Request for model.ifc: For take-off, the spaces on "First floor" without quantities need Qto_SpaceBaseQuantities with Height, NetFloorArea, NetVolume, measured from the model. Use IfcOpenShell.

First a look at what the model holds.

```python
import ifcopenshell
import ifcopenshell.util.element
import ifcopenshell.util.unit

model = ifcopenshell.open("model.ifc")
print(model.schema)
for unit_type in ("LENGTHUNIT", "AREAUNIT", "VOLUMEUNIT"):
    print(unit_type, ifcopenshell.util.unit.calculate_unit_scale(model, unit_type))
storey = next(s for s in model.by_type("IfcBuildingStorey") if s.Name == "First floor")
spaces = [e for e in ifcopenshell.util.element.get_decomposition(storey) if e.is_a("IfcSpace")]
for e in sorted(spaces, key=lambda e: e.id()):
    print(e.id(), e.is_a(), e.Name, list(ifcopenshell.util.element.get_psets(e, qtos_only=True)), sep=" | ")
```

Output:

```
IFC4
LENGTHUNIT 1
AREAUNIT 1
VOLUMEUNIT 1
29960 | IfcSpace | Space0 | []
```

```python
import ifcopenshell
import ifcopenshell.api.pset
import ifcopenshell.geom
import ifcopenshell.util.element
import ifcopenshell.util.shape
import ifcopenshell.util.unit

model = ifcopenshell.open("model.ifc")
unit_scale = ifcopenshell.util.unit.calculate_unit_scale(model)
area_scale = ifcopenshell.util.unit.calculate_unit_scale(model, "AREAUNIT")
volume_scale = ifcopenshell.util.unit.calculate_unit_scale(model, "VOLUMEUNIT")
settings = ifcopenshell.geom.settings()

storey = next(s for s in model.by_type("IfcBuildingStorey") if s.Name == "First floor")
spaces = [e for e in ifcopenshell.util.element.get_decomposition(storey) if e.is_a("IfcSpace")]

for e in sorted(spaces, key=lambda e: e.id()):
    if ifcopenshell.util.element.get_psets(e, qtos_only=True, should_inherit=False):
        continue
    # Geometry comes back in metres, in the element's own axes.
    shape = ifcopenshell.geom.create_shape(settings, e)
    values = {
        "Height": ifcopenshell.util.shape.get_z(shape.geometry) / unit_scale,
        "NetFloorArea": ifcopenshell.util.shape.get_footprint_area(shape.geometry) / area_scale,
        "NetVolume": ifcopenshell.util.shape.get_volume(shape.geometry) / volume_scale,
    }
    qto = ifcopenshell.api.pset.add_qto(model, product=e, name="Qto_SpaceBaseQuantities")
    ifcopenshell.api.pset.edit_qto(model, qto=qto, properties=values)
    print(e.id(), {k: round(v, 3) for k, v in values.items()})

model.write("model_v2.ifc")
```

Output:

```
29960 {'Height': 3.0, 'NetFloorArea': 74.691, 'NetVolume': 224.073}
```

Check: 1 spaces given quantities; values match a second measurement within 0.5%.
